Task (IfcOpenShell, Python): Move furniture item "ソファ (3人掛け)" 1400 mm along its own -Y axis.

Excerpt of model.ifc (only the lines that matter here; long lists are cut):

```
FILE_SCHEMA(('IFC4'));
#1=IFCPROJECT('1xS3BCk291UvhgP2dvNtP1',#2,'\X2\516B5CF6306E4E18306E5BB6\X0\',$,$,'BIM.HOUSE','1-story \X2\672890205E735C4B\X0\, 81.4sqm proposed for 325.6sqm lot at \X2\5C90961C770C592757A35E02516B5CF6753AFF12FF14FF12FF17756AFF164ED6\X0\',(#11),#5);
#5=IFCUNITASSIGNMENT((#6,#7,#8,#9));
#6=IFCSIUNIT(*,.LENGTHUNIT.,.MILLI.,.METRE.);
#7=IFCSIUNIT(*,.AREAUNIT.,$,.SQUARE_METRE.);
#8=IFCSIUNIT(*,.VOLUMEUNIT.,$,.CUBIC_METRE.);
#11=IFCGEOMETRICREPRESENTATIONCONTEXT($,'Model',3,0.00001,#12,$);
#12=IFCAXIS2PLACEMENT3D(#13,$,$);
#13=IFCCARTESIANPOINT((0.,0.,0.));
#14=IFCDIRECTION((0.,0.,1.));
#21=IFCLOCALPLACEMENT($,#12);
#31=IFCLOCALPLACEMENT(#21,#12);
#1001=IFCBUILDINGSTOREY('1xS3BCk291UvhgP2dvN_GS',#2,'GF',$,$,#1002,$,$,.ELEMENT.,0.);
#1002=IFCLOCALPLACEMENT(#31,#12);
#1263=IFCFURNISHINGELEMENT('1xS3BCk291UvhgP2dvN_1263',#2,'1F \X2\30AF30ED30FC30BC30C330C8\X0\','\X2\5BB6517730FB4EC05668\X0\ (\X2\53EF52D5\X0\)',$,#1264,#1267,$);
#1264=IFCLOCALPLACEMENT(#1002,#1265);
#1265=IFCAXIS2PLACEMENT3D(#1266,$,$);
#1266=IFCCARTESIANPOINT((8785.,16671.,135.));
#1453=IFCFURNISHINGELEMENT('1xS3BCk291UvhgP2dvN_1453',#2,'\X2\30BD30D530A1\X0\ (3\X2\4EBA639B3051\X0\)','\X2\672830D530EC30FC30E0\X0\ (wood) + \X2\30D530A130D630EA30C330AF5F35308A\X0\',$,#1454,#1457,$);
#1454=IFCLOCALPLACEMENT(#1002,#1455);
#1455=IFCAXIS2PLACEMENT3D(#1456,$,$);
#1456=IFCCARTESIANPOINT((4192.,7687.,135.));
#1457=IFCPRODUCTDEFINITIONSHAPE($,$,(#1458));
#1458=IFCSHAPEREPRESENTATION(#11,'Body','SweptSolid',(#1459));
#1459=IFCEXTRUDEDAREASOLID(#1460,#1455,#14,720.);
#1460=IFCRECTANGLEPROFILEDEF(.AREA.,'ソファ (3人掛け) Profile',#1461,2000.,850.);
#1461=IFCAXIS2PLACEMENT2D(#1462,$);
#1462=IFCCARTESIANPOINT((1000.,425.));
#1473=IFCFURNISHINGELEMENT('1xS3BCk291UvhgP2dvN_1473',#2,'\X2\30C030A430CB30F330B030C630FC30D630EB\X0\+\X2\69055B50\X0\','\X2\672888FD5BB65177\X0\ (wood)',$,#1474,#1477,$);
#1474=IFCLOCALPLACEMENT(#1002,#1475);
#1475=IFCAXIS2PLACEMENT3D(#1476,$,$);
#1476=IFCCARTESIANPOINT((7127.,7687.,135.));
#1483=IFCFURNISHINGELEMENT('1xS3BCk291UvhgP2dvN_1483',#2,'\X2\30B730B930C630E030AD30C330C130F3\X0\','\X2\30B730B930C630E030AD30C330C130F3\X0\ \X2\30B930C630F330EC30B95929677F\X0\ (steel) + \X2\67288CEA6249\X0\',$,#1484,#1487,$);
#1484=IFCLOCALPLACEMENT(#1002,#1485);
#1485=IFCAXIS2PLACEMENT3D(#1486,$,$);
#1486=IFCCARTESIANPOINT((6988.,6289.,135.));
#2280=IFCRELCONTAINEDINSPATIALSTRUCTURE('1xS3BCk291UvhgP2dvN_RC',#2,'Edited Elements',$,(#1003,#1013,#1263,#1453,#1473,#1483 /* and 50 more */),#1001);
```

```python
import ifcopenshell
import ifcopenshell.api.geometry
import ifcopenshell.util.placement

model = ifcopenshell.open("model.ifc")

item = model.by_guid("1xS3BCk291UvhgP2dvN_1453")
matrix = ifcopenshell.util.placement.get_local_placement(item.ObjectPlacement)
matrix[:3, 3] -= matrix[:3, 1] * 1400.0
ifcopenshell.api.geometry.edit_object_placement(model, product=item, matrix=matrix, is_si=False)

print(ifcopenshell.util.placement.get_local_placement(item.ObjectPlacement).round(3) + 0.0)

model.write("model_v2.ifc")
```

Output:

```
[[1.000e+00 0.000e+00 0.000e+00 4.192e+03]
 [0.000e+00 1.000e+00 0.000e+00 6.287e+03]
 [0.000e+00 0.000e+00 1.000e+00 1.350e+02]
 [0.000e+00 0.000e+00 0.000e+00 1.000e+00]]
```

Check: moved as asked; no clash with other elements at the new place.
